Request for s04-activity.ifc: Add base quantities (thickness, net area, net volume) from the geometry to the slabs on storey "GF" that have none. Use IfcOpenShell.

First a look at what the model holds.

```python
import ifcopenshell
import ifcopenshell.util.element
import ifcopenshell.util.unit

model = ifcopenshell.open("s04-activity.ifc")
print(model.schema)
for unit_type in ("LENGTHUNIT", "AREAUNIT", "VOLUMEUNIT"):
    print(unit_type, ifcopenshell.util.unit.calculate_unit_scale(model, unit_type))
storey = next(s for s in model.by_type("IfcBuildingStorey") if s.Name == "GF")
slabs = [e for e in ifcopenshell.util.element.get_decomposition(storey) if e.is_a("IfcSlab")]
for e in sorted(slabs, key=lambda e: e.id()):
    print(e.id(), e.is_a(), e.Name, list(ifcopenshell.util.element.get_psets(e, qtos_only=True)), sep=" | ")
```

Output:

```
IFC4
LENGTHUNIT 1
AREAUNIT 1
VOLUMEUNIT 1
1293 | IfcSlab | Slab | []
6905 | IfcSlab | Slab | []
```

```python
import ifcopenshell
import ifcopenshell.api.pset
import ifcopenshell.geom
import ifcopenshell.util.element
import ifcopenshell.util.shape
import ifcopenshell.util.unit

model = ifcopenshell.open("s04-activity.ifc")
unit_scale = ifcopenshell.util.unit.calculate_unit_scale(model)
area_scale = ifcopenshell.util.unit.calculate_unit_scale(model, "AREAUNIT")
volume_scale = ifcopenshell.util.unit.calculate_unit_scale(model, "VOLUMEUNIT")
settings = ifcopenshell.geom.settings()

storey = next(s for s in model.by_type("IfcBuildingStorey") if s.Name == "GF")
slabs = [e for e in ifcopenshell.util.element.get_decomposition(storey) if e.is_a("IfcSlab")]

for e in sorted(slabs, key=lambda e: e.id()):
    if ifcopenshell.util.element.get_psets(e, qtos_only=True, should_inherit=False):
        continue
    # Geometry comes back in metres, in the element's own axes.
    shape = ifcopenshell.geom.create_shape(settings, e)
    values = {
        "Width": ifcopenshell.util.shape.get_z(shape.geometry) / unit_scale,
        "NetArea": ifcopenshell.util.shape.get_footprint_area(shape.geometry) / area_scale,
        "NetVolume": ifcopenshell.util.shape.get_volume(shape.geometry) / volume_scale,
    }
    qto = ifcopenshell.api.pset.add_qto(model, product=e, name="Qto_SlabBaseQuantities")
    ifcopenshell.api.pset.edit_qto(model, qto=qto, properties=values)
    print(e.id(), {k: round(v, 3) for k, v in values.items()})

model.write("s04-activity_v2.ifc")
```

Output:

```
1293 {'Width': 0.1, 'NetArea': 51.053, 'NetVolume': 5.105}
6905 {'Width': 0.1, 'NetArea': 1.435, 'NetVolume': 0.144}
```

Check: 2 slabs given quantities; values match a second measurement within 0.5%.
